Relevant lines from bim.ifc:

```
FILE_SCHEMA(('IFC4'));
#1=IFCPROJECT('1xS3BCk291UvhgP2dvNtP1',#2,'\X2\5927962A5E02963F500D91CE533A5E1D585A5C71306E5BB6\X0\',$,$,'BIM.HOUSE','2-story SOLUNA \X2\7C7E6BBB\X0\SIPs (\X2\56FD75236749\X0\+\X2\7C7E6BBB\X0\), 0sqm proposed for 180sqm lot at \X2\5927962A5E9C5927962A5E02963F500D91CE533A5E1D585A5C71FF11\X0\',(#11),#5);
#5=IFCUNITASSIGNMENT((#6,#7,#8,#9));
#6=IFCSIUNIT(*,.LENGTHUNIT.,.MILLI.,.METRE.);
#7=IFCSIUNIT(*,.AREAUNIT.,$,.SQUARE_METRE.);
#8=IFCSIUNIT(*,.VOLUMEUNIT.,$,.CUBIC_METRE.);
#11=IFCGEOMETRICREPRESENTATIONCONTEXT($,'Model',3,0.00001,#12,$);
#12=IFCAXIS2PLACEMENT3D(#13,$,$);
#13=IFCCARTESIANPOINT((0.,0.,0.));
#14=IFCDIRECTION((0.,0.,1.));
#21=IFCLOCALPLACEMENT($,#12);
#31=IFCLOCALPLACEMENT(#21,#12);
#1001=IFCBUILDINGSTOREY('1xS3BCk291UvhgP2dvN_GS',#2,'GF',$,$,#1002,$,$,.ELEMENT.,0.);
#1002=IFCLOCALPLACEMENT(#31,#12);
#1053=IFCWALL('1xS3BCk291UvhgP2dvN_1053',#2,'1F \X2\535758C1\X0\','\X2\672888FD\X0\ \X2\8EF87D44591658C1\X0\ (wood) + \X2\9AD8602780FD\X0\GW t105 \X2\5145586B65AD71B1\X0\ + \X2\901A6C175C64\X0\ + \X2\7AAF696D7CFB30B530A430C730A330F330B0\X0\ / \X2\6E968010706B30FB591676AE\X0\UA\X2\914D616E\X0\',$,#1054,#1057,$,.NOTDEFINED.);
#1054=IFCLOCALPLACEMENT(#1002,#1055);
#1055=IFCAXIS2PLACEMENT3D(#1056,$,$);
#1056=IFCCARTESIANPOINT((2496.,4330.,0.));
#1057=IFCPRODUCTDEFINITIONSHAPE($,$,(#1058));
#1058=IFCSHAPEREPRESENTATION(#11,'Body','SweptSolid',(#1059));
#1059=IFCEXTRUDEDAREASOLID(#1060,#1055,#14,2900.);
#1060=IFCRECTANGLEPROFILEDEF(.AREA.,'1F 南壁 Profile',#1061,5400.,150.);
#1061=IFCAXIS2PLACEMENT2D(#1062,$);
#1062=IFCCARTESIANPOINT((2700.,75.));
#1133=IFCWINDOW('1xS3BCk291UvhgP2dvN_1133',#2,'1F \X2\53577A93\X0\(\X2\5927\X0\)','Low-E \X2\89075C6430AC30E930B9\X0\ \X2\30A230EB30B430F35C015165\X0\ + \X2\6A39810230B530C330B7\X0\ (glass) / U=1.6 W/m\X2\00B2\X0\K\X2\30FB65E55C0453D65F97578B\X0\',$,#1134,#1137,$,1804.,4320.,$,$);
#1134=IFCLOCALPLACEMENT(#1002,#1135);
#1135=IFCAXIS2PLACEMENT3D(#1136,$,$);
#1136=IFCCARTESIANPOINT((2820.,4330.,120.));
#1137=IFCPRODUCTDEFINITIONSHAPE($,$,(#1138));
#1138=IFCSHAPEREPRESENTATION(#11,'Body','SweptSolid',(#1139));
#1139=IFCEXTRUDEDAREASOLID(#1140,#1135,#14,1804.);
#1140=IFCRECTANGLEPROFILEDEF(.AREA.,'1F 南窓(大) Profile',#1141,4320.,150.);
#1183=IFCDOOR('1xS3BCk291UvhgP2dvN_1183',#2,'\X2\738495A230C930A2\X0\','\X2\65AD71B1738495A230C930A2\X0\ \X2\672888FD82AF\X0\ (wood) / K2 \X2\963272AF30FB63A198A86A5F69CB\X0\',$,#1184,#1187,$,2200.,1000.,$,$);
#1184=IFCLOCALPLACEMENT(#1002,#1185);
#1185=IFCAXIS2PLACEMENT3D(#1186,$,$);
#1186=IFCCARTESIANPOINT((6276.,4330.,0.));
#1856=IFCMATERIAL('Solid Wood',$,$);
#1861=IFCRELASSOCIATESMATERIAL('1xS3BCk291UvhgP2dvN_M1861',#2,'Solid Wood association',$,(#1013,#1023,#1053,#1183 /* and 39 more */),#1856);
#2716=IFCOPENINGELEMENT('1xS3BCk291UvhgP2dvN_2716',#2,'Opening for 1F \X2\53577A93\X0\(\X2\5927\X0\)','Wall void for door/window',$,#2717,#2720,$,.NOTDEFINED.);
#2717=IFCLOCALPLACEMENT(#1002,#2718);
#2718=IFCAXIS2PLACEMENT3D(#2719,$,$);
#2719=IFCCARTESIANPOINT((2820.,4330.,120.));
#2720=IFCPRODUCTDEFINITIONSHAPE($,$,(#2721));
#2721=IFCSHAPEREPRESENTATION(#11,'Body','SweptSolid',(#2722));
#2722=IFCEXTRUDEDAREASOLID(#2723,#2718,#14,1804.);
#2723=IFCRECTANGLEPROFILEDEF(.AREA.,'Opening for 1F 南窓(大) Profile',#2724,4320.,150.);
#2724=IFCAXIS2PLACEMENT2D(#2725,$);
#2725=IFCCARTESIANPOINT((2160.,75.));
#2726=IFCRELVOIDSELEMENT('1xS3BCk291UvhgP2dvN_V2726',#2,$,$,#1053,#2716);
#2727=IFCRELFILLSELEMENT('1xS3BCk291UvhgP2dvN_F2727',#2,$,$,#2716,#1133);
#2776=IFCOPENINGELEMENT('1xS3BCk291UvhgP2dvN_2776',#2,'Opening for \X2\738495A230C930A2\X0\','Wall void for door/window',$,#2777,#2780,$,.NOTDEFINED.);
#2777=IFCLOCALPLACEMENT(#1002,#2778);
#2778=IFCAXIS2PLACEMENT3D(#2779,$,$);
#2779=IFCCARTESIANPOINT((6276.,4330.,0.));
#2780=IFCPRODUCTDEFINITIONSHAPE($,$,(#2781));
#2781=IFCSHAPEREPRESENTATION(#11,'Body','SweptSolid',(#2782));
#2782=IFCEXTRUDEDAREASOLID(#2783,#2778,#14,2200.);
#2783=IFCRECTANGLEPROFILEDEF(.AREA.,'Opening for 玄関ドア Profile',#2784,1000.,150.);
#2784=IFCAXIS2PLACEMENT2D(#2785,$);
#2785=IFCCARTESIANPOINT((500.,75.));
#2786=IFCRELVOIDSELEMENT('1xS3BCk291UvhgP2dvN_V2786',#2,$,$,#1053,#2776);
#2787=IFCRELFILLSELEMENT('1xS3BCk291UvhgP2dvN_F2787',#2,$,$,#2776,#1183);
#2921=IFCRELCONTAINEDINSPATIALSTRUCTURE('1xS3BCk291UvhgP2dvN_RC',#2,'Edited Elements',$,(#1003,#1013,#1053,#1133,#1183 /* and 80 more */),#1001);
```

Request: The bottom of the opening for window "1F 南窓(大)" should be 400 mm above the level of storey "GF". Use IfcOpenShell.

```python
import numpy as np
import ifcopenshell
import ifcopenshell.api.geometry
import ifcopenshell.geom
import ifcopenshell.util.element
import ifcopenshell.util.placement
import ifcopenshell.util.shape
import ifcopenshell.util.unit

model = ifcopenshell.open("bim.ifc")
unit_scale = ifcopenshell.util.unit.calculate_unit_scale(model)

window = model.by_id(1133)
opening = window.FillsVoids[0].RelatingOpeningElement
storey = ifcopenshell.util.element.get_container(window, ifc_class="IfcBuildingStorey")
level = ifcopenshell.util.placement.get_local_placement(storey.ObjectPlacement)[2, 3]

# The opening's origin need not be at the sill, so measure its lowest point.
shape = ifcopenshell.geom.create_shape(ifcopenshell.geom.settings(), opening)
bottom = ifcopenshell.util.shape.get_shape_bottom_elevation(shape, shape.geometry) / unit_scale
dz = level + 0.4 / unit_scale - bottom

shift = np.array([0.0, 0.0, dz])
# The window is not placed relative to its opening, so move both.
for product in (opening, window):
    matrix = ifcopenshell.util.placement.get_local_placement(product.ObjectPlacement)
    matrix[:3, 3] += shift
    ifcopenshell.api.geometry.edit_object_placement(model, product=product, matrix=matrix, is_si=False)

print(f"moved by {dz * unit_scale:+.3f} m")

model.write("bim_rev.ifc")
```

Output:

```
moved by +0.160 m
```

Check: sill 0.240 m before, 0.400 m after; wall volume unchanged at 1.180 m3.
